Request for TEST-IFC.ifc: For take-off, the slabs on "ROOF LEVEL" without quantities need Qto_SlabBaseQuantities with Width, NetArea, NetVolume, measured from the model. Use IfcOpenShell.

First a look at what the model holds.

```python
import ifcopenshell
import ifcopenshell.util.element
import ifcopenshell.util.unit

model = ifcopenshell.open("TEST-IFC.ifc")
print(model.schema)
for unit_type in ("LENGTHUNIT", "AREAUNIT", "VOLUMEUNIT"):
    print(unit_type, ifcopenshell.util.unit.calculate_unit_scale(model, unit_type))
storey = next(s for s in model.by_type("IfcBuildingStorey") if s.Name == "ROOF LEVEL")
slabs = [e for e in ifcopenshell.util.element.get_decomposition(storey) if e.is_a("IfcSlab")]
for e in sorted(slabs, key=lambda e: e.id()):
    print(e.id(), e.is_a(), e.Name, list(ifcopenshell.util.element.get_psets(e, qtos_only=True)), sep=" | ")
```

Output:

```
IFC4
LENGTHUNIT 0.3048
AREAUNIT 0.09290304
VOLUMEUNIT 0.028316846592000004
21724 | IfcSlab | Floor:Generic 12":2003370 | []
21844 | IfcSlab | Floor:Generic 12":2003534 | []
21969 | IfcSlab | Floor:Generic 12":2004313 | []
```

```python
import ifcopenshell
import ifcopenshell.api.pset
import ifcopenshell.geom
import ifcopenshell.util.element
import ifcopenshell.util.shape
import ifcopenshell.util.unit

model = ifcopenshell.open("TEST-IFC.ifc")
unit_scale = ifcopenshell.util.unit.calculate_unit_scale(model)
area_scale = ifcopenshell.util.unit.calculate_unit_scale(model, "AREAUNIT")
volume_scale = ifcopenshell.util.unit.calculate_unit_scale(model, "VOLUMEUNIT")
settings = ifcopenshell.geom.settings()

storey = next(s for s in model.by_type("IfcBuildingStorey") if s.Name == "ROOF LEVEL")
slabs = [e for e in ifcopenshell.util.element.get_decomposition(storey) if e.is_a("IfcSlab")]

for e in sorted(slabs, key=lambda e: e.id()):
    if ifcopenshell.util.element.get_psets(e, qtos_only=True, should_inherit=False):
        continue
    # Geometry comes back in metres, in the element's own axes.
    shape = ifcopenshell.geom.create_shape(settings, e)
    values = {
        "Width": ifcopenshell.util.shape.get_z(shape.geometry) / unit_scale,
        "NetArea": ifcopenshell.util.shape.get_footprint_area(shape.geometry) / area_scale,
        "NetVolume": ifcopenshell.util.shape.get_volume(shape.geometry) / volume_scale,
    }
    qto = ifcopenshell.api.pset.add_qto(model, product=e, name="Qto_SlabBaseQuantities")
    ifcopenshell.api.pset.edit_qto(model, qto=qto, properties=values)
    print(e.id(), {k: round(v, 3) for k, v in values.items()})

model.write("TEST-IFC_updated.ifc")
```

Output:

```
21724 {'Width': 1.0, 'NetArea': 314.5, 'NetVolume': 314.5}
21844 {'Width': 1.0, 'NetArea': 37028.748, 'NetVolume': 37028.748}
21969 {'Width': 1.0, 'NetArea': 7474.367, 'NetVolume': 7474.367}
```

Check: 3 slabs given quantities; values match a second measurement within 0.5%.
